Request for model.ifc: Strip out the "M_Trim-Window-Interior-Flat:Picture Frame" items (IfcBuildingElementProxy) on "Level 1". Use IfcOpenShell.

First a look at what the model holds.

```python
import ifcopenshell
import ifcopenshell.util.element

model = ifcopenshell.open("model.ifc")
print(model.schema)
storey = next(s for s in model.by_type("IfcBuildingStorey") if s.Name == "Level 1")
proxies = [e for e in ifcopenshell.util.element.get_decomposition(storey) if e.is_a("IfcBuildingElementProxy")]
seen = {}
for e in proxies:
    element_type = ifcopenshell.util.element.get_type(e)
    name = element_type.Name if element_type not in (None, e) else None
    seen[name] = seen.get(name, 0) + 1
for name, count in sorted(seen.items(), key=str):
    print(count, "x", name)
```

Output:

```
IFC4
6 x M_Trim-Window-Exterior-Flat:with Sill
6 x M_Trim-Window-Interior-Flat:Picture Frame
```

```python
import ifcopenshell
import ifcopenshell.api.root
import ifcopenshell.util.element

model = ifcopenshell.open("model.ifc")

storey = next(s for s in model.by_type("IfcBuildingStorey") if s.Name == "Level 1")
proxies = [e for e in ifcopenshell.util.element.get_decomposition(storey) if e.is_a("IfcBuildingElementProxy")]
targets = [e for e in proxies if (t := ifcopenshell.util.element.get_type(e)) not in (None, e) and t.Name == "M_Trim-Window-Interior-Flat:Picture Frame"]

for e in targets:
    ifcopenshell.api.root.remove_product(model, product=e)
print(len(targets), "removed")

model.write("model-out.ifc")
```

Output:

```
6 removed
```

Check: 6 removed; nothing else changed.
